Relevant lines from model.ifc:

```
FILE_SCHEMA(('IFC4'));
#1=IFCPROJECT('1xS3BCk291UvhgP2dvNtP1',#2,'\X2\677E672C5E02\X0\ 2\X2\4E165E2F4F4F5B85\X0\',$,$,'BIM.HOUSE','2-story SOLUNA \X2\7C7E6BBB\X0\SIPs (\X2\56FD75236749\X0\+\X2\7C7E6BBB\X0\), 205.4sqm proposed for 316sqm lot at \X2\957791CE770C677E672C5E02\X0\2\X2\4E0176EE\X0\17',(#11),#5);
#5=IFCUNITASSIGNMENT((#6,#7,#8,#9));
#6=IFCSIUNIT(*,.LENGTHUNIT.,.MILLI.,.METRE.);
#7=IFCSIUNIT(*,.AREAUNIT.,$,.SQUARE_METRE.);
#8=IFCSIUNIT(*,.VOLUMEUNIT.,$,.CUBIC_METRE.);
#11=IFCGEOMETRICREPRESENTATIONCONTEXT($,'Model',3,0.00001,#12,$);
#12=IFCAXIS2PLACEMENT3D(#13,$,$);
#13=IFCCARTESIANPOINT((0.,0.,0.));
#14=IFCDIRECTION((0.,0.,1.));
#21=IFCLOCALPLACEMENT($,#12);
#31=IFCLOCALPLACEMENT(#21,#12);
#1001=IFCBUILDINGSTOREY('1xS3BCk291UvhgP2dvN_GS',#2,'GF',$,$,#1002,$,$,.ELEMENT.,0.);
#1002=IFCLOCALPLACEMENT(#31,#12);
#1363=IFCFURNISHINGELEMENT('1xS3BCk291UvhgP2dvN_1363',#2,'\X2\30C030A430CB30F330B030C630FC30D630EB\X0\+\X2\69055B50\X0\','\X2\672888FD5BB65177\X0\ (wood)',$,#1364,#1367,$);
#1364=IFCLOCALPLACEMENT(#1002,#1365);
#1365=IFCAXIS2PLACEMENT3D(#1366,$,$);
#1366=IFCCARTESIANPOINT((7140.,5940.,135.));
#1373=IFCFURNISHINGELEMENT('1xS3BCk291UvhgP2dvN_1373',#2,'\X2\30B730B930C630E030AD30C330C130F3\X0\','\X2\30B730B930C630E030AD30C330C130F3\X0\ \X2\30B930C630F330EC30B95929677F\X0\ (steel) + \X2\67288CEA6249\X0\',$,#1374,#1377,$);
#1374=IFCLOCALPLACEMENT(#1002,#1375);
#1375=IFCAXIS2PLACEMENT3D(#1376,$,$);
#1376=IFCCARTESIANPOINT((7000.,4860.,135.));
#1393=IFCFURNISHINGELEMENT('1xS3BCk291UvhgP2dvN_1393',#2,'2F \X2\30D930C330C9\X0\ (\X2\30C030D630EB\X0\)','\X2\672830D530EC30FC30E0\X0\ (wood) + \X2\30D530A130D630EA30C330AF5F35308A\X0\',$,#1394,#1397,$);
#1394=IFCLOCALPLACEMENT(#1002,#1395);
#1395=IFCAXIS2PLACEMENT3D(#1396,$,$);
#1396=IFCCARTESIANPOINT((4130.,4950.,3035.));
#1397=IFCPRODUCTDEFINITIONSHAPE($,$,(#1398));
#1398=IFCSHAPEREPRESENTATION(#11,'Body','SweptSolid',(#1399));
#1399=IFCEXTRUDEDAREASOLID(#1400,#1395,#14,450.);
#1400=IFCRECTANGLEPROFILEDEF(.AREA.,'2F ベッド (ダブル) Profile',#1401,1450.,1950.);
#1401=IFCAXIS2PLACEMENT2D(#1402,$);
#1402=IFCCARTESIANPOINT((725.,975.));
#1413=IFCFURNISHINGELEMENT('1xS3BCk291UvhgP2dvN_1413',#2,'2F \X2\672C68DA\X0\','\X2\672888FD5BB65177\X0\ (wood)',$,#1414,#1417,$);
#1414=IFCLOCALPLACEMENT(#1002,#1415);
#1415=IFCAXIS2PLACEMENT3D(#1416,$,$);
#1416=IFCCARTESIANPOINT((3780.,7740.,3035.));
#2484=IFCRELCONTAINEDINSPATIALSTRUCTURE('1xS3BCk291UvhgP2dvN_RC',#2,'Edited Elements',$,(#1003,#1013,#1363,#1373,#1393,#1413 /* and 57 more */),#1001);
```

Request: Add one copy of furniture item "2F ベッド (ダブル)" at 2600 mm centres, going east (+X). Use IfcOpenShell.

```python
import numpy as np
import ifcopenshell
import ifcopenshell.api.geometry
import ifcopenshell.api.root
import ifcopenshell.util.element
import ifcopenshell.util.placement
import ifcopenshell.util.unit

model = ifcopenshell.open("model.ifc")
unit_scale = ifcopenshell.util.unit.calculate_unit_scale(model)


def reuse_history(source, copy):
    """copy_class also copies each property set's owner history, people and application; keep the originals."""
    for rel in copy.IsDefinedBy:
        if rel.is_a("IfcRelDefinesByProperties") and (history := rel.RelatingPropertyDefinition.OwnerHistory):
            rel.RelatingPropertyDefinition.OwnerHistory = source.OwnerHistory
            ifcopenshell.util.element.remove_deep2(model, history)


source = model.by_guid("1xS3BCk291UvhgP2dvN_1393")
base = ifcopenshell.util.placement.get_local_placement(source.ObjectPlacement)
step = np.array([1.0, 0.0, 0.0]) * 2.6 / unit_scale

for i in range(1, 2):
    copy = ifcopenshell.api.root.copy_class(model, product=source)
    copy.Representation = ifcopenshell.util.element.copy_deep(
        model, source.Representation, exclude=["IfcGeometricRepresentationContext", "IfcRepresentationMap"]
    )
    reuse_history(source, copy)
    matrix = base.copy()
    matrix[:3, 3] += i * step
    print("added at", matrix[:3, 3].round(3) + 0.0)
    ifcopenshell.api.geometry.edit_object_placement(model, product=copy, matrix=matrix, is_si=False)

model.write("model_rev.ifc")
```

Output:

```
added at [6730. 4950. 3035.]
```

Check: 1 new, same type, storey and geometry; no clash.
